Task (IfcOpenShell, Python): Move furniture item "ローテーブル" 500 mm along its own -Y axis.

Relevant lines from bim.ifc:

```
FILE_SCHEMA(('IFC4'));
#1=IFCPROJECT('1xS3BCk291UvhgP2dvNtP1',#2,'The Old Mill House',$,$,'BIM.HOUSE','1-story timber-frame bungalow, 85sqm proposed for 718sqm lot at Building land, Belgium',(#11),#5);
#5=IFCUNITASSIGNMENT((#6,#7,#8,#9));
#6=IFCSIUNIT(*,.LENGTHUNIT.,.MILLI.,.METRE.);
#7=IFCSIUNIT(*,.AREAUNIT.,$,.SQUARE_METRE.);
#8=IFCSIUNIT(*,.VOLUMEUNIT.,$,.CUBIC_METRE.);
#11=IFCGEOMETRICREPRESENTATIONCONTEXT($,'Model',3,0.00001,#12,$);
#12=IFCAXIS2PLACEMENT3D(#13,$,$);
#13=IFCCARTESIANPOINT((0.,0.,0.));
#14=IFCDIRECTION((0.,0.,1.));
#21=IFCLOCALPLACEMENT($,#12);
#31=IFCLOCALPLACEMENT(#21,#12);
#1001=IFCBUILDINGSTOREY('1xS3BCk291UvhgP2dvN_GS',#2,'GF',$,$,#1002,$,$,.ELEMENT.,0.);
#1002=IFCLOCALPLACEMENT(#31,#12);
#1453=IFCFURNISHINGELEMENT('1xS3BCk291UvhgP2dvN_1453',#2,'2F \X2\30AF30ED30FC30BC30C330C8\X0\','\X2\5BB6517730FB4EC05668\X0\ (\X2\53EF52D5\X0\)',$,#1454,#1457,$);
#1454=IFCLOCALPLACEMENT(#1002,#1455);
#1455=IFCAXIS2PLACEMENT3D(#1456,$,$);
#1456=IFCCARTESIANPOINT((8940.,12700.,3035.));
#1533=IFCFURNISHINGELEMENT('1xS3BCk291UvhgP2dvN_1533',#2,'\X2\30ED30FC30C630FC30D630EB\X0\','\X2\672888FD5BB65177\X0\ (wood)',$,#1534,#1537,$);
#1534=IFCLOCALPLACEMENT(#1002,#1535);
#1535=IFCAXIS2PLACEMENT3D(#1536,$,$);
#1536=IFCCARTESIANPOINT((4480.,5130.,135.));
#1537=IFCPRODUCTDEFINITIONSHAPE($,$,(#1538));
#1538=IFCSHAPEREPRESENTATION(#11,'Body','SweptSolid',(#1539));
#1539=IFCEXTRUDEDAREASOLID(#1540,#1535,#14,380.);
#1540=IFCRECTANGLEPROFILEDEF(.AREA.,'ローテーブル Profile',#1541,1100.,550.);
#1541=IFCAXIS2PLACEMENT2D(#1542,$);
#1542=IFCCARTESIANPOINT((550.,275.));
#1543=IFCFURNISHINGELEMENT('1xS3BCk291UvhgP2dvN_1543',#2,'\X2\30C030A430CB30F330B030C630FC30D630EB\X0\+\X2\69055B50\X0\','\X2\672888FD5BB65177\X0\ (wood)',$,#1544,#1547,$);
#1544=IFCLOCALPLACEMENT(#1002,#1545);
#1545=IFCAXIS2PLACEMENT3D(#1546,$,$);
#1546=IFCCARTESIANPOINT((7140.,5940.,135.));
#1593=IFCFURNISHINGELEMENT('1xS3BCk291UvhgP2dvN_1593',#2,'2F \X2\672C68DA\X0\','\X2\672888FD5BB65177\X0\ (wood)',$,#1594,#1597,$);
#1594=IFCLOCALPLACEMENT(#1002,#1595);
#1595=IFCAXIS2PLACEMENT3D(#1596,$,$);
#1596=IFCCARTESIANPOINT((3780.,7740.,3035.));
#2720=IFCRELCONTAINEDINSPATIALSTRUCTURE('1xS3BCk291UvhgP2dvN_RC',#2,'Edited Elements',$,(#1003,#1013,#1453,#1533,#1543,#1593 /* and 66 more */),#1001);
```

```python
import ifcopenshell
import ifcopenshell.api.geometry
import ifcopenshell.util.placement

model = ifcopenshell.open("bim.ifc")

item = model.by_guid("1xS3BCk291UvhgP2dvN_1533")
matrix = ifcopenshell.util.placement.get_local_placement(item.ObjectPlacement)
matrix[:3, 3] -= matrix[:3, 1] * 500.0
ifcopenshell.api.geometry.edit_object_placement(model, product=item, matrix=matrix, is_si=False)

print(ifcopenshell.util.placement.get_local_placement(item.ObjectPlacement).round(3) + 0.0)

model.write("bim_rev.ifc")
```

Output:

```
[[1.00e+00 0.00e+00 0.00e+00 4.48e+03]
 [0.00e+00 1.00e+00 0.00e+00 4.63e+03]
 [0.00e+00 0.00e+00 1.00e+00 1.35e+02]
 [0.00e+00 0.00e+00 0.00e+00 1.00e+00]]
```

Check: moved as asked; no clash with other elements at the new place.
